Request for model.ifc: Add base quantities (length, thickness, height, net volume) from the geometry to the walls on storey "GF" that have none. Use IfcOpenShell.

First a look at what the model holds.

```python
import ifcopenshell
import ifcopenshell.util.element
import ifcopenshell.util.unit

model = ifcopenshell.open("model.ifc")
print(model.schema)
for unit_type in ("LENGTHUNIT", "AREAUNIT", "VOLUMEUNIT"):
    print(unit_type, ifcopenshell.util.unit.calculate_unit_scale(model, unit_type))
storey = next(s for s in model.by_type("IfcBuildingStorey") if s.Name == "GF")
walls = [e for e in ifcopenshell.util.element.get_decomposition(storey) if e.is_a("IfcWall")]
for e in sorted(walls, key=lambda e: e.id()):
    print(e.id(), e.is_a(), e.Name, list(ifcopenshell.util.element.get_psets(e, qtos_only=True)), sep=" | ")
```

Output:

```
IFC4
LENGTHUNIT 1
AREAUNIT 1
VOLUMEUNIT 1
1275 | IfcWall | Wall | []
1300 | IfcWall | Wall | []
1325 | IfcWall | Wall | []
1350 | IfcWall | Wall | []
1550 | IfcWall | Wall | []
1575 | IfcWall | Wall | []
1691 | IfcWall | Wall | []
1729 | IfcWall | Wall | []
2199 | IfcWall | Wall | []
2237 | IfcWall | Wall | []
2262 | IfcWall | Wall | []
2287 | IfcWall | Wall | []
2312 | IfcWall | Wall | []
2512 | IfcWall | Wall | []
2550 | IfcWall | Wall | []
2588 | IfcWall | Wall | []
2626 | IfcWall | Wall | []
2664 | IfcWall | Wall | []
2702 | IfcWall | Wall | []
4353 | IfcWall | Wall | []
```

```python
import ifcopenshell
import ifcopenshell.api.pset
import ifcopenshell.geom
import ifcopenshell.util.element
import ifcopenshell.util.shape
import ifcopenshell.util.unit

model = ifcopenshell.open("model.ifc")
unit_scale = ifcopenshell.util.unit.calculate_unit_scale(model)
volume_scale = ifcopenshell.util.unit.calculate_unit_scale(model, "VOLUMEUNIT")
settings = ifcopenshell.geom.settings()

storey = next(s for s in model.by_type("IfcBuildingStorey") if s.Name == "GF")
walls = [e for e in ifcopenshell.util.element.get_decomposition(storey) if e.is_a("IfcWall")]

for e in sorted(walls, key=lambda e: e.id()):
    if ifcopenshell.util.element.get_psets(e, qtos_only=True, should_inherit=False):
        continue
    # Geometry comes back in metres, in the element's own axes.
    shape = ifcopenshell.geom.create_shape(settings, e)
    values = {
        "Length": ifcopenshell.util.shape.get_x(shape.geometry) / unit_scale,
        "Width": ifcopenshell.util.shape.get_y(shape.geometry) / unit_scale,
        "Height": ifcopenshell.util.shape.get_z(shape.geometry) / unit_scale,
        "NetVolume": ifcopenshell.util.shape.get_volume(shape.geometry) / volume_scale,
    }
    qto = ifcopenshell.api.pset.add_qto(model, product=e, name="Qto_WallBaseQuantities")
    ifcopenshell.api.pset.edit_qto(model, qto=qto, properties=values)
    print(e.id(), {k: round(v, 3) for k, v in values.items()})

model.write("model_rev.ifc")
```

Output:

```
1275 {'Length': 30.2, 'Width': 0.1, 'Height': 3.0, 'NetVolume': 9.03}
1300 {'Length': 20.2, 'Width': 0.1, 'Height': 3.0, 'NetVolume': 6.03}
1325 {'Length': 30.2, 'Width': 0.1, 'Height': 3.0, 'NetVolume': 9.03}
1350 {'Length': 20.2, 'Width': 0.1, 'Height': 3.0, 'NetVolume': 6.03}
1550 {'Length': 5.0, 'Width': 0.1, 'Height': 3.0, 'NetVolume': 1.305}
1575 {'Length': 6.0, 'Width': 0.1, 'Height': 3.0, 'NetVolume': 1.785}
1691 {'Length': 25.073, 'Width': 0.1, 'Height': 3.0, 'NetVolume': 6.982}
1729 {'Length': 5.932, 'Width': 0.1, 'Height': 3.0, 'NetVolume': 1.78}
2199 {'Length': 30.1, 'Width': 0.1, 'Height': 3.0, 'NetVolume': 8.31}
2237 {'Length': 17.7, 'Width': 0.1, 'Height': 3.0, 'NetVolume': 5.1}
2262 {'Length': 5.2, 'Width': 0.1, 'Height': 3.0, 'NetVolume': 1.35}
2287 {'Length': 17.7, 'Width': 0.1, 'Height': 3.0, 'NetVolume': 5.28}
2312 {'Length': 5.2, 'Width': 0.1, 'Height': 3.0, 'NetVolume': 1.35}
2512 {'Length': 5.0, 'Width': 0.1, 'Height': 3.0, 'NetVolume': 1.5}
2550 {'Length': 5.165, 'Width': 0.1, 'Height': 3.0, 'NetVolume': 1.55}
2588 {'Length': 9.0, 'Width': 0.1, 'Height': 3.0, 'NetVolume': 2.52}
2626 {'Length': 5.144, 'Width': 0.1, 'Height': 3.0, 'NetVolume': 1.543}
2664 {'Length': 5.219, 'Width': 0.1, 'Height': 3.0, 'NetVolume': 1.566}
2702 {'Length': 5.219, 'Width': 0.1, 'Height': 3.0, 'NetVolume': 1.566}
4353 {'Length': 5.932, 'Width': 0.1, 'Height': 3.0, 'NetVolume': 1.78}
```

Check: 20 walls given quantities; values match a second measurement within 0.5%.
